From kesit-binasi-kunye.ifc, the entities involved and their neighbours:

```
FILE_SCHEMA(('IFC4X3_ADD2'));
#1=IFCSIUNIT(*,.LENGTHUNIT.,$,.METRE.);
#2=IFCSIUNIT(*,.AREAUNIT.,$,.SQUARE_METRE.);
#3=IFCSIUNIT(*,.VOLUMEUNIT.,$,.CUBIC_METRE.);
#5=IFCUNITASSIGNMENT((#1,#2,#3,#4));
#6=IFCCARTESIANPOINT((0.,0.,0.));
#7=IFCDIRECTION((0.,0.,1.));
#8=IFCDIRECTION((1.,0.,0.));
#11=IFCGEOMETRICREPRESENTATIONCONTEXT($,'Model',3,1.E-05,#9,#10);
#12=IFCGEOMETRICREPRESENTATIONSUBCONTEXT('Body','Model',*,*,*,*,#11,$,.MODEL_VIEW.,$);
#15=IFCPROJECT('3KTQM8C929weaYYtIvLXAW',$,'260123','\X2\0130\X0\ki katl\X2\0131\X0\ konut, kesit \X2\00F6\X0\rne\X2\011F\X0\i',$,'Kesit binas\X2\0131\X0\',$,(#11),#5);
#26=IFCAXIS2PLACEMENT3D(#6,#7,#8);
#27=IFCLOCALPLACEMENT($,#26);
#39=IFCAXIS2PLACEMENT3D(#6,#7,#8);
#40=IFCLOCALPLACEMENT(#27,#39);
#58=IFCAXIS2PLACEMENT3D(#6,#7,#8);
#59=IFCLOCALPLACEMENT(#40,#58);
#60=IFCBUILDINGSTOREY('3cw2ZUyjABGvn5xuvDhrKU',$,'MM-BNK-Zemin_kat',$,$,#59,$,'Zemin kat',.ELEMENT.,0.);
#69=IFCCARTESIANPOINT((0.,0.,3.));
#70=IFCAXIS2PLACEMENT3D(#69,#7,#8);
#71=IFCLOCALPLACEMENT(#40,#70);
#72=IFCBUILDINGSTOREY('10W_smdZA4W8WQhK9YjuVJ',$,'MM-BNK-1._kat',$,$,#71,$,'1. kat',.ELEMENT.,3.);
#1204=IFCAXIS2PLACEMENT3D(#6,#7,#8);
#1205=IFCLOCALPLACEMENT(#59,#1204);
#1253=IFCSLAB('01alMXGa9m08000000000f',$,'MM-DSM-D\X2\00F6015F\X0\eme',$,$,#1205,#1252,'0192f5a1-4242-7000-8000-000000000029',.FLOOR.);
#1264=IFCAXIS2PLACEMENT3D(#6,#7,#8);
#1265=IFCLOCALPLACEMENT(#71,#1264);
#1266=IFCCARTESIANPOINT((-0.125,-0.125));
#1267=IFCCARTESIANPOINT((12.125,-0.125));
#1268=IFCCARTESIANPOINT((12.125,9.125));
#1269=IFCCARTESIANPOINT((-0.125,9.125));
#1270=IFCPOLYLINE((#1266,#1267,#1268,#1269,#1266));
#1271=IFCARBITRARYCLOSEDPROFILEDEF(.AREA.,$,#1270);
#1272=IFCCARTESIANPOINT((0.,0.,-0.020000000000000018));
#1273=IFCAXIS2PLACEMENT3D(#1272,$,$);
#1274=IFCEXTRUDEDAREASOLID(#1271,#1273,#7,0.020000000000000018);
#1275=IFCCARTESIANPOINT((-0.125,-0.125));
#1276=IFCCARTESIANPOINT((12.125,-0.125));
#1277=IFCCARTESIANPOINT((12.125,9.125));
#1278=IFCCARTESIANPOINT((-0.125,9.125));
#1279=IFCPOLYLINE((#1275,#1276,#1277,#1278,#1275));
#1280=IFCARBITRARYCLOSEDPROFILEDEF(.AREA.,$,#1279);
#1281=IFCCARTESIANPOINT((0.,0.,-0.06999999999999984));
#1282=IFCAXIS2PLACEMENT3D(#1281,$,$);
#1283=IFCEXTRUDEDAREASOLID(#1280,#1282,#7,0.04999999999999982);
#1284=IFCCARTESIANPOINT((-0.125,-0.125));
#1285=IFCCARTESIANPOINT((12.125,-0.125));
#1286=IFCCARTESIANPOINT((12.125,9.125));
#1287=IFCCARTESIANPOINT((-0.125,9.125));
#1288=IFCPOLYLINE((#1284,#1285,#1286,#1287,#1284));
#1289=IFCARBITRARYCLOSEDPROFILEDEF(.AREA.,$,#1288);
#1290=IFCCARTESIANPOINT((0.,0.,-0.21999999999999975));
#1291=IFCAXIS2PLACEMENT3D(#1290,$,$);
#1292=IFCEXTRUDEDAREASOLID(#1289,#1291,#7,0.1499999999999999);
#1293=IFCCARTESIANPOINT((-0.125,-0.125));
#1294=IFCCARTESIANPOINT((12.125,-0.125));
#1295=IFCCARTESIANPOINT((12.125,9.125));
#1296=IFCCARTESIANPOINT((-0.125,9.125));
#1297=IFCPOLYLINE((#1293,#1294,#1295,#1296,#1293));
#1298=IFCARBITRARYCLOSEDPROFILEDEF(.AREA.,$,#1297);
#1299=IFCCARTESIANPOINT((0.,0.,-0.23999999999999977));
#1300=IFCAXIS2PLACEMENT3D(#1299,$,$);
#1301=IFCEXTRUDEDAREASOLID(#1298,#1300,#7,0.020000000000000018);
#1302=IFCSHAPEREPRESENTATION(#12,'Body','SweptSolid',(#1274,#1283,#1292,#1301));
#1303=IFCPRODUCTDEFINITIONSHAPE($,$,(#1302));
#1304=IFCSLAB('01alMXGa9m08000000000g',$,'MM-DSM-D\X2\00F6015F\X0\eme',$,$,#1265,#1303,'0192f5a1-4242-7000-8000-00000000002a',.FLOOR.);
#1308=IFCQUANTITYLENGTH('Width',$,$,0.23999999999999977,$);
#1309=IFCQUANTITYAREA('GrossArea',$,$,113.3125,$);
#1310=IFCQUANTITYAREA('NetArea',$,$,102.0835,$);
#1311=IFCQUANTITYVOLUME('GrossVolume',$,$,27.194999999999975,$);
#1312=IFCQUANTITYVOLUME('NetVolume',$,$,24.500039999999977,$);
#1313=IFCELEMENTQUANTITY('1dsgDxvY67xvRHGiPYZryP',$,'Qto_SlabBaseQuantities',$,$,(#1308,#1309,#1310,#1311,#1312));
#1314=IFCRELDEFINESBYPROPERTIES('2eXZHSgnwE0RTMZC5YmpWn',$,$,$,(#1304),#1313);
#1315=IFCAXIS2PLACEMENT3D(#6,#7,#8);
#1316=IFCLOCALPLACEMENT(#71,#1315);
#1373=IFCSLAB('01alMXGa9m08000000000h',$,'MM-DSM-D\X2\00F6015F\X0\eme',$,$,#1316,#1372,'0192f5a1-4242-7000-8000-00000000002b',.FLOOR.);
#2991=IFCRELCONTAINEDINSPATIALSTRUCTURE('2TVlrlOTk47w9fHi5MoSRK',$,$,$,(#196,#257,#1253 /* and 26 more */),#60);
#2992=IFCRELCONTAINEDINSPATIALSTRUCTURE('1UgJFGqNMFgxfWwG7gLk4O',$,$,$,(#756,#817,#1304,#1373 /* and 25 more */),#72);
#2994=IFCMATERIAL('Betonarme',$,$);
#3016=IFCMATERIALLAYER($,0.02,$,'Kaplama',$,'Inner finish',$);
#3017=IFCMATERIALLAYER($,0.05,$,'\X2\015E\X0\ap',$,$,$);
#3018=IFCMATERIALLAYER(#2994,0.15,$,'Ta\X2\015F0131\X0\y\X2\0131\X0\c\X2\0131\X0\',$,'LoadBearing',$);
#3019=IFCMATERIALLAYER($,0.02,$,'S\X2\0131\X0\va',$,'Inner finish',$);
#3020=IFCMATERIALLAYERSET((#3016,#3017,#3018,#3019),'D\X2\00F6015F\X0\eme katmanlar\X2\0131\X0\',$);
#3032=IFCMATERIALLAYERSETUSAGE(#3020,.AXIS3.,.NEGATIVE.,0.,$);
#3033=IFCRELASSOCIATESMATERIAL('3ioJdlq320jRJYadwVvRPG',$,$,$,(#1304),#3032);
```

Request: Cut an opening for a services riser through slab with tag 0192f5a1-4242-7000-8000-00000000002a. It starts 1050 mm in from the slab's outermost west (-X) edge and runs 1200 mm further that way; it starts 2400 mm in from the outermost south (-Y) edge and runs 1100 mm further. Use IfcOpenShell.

```python
import numpy as np
import ifcopenshell
import ifcopenshell.api.feature
import ifcopenshell.api.geometry
import ifcopenshell.api.pset
import ifcopenshell.api.root
import ifcopenshell.geom
import ifcopenshell.util.element
import ifcopenshell.util.placement
import ifcopenshell.util.representation
import ifcopenshell.util.shape
import ifcopenshell.util.unit

model = ifcopenshell.open("kesit-binasi-kunye.ifc")
unit_scale = ifcopenshell.util.unit.calculate_unit_scale(model)
area_scale = ifcopenshell.util.unit.calculate_unit_scale(model, "AREAUNIT")
volume_scale = ifcopenshell.util.unit.calculate_unit_scale(model, "VOLUMEUNIT")
settings = ifcopenshell.geom.settings()


def volume(element):
    """Net volume in cubic metres, openings subtracted."""
    shape = ifcopenshell.geom.create_shape(settings, element)
    return ifcopenshell.util.shape.get_volume(shape.geometry)


slab = model.by_guid("01alMXGa9m08000000000g")
before = volume(slab)

# Extent in the slab's own axes, in metres. The edges named are its -X and -Y sides.
slab_shape = ifcopenshell.geom.create_shape(settings, slab)
vertices = ifcopenshell.util.shape.get_vertices(slab_shape.geometry)
x_min, y_min, bottom = vertices.min(axis=0)
top = vertices[:, 2].max()

opening = ifcopenshell.api.root.create_entity(model, ifc_class="IfcOpeningElement", name="Services riser opening", predefined_type="OPENING")
context = ifcopenshell.util.representation.get_context(model, "Model", "Body", "MODEL_VIEW")
width, depth = 1.2, 1.1
outline = [(0.0, 0.0), (width, 0.0), (width, depth), (0.0, depth), (0.0, 0.0)]
# Overshoot both faces by 50 mm so the cut is clean.
shape = ifcopenshell.api.geometry.add_slab_representation(
    model, context=context, depth=top - bottom + 0.1, polyline=outline
)
ifcopenshell.api.geometry.assign_representation(model, product=opening, representation=shape)

matrix = ifcopenshell.util.placement.get_local_placement(slab.ObjectPlacement)
matrix[:, 3] = matrix @ np.append(np.array([x_min + 1.05, y_min + 2.4, bottom - 0.05]) / unit_scale, 1.0)
ifcopenshell.api.geometry.edit_object_placement(model, product=opening, matrix=matrix, is_si=False)
ifcopenshell.api.feature.add_feature(model, feature=opening, element=slab)

after = volume(slab)

# Update the slab's stored quantities.
qto = model.by_id(ifcopenshell.util.element.get_pset(slab, "Qto_SlabBaseQuantities", should_inherit=False)["id"])
ifcopenshell.api.pset.edit_qto(model, qto=qto, properties={
    "NetArea": after / (top - bottom) / area_scale,
    "NetVolume": after / volume_scale,
})

print(f"slab volume {before:.3f} -> {after:.3f} m3")

model.write("kesit-binasi-kunye_rev.ifc")
```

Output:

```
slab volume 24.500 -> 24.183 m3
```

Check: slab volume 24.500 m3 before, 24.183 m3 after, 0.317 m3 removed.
